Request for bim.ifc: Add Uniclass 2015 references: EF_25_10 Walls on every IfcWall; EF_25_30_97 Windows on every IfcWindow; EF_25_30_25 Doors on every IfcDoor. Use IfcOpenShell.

First a look at what the model holds.

```python
import ifcopenshell

model = ifcopenshell.open("bim.ifc")
print(model.schema)
print("classifications:", [c.Name for c in model.by_type("IfcClassification")])
for ifc_class in ("IfcDoor", "IfcRoof", "IfcStair", "IfcWall", "IfcWindow"):
    print(ifc_class, len(model.by_type(ifc_class)))
```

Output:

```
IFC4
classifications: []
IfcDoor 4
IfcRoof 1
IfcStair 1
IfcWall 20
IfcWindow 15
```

```python
import ifcopenshell
import ifcopenshell.api.classification

model = ifcopenshell.open("bim.ifc")

system = ifcopenshell.api.classification.add_classification(model, classification="Uniclass 2015")

codes = {
    "IfcWall": ("EF_25_10", "Walls"),
    "IfcWindow": ("EF_25_30_97", "Windows"),
    "IfcDoor": ("EF_25_30_25", "Doors"),
}
for ifc_class, (code, name) in codes.items():
    products = model.by_type(ifc_class)
    ifcopenshell.api.classification.add_reference(
        model, products=products, classification=system, identification=code, name=name
    )
    print(code, len(products))

model.write("bim_rev.ifc")
```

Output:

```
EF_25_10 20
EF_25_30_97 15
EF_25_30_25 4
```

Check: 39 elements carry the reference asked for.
